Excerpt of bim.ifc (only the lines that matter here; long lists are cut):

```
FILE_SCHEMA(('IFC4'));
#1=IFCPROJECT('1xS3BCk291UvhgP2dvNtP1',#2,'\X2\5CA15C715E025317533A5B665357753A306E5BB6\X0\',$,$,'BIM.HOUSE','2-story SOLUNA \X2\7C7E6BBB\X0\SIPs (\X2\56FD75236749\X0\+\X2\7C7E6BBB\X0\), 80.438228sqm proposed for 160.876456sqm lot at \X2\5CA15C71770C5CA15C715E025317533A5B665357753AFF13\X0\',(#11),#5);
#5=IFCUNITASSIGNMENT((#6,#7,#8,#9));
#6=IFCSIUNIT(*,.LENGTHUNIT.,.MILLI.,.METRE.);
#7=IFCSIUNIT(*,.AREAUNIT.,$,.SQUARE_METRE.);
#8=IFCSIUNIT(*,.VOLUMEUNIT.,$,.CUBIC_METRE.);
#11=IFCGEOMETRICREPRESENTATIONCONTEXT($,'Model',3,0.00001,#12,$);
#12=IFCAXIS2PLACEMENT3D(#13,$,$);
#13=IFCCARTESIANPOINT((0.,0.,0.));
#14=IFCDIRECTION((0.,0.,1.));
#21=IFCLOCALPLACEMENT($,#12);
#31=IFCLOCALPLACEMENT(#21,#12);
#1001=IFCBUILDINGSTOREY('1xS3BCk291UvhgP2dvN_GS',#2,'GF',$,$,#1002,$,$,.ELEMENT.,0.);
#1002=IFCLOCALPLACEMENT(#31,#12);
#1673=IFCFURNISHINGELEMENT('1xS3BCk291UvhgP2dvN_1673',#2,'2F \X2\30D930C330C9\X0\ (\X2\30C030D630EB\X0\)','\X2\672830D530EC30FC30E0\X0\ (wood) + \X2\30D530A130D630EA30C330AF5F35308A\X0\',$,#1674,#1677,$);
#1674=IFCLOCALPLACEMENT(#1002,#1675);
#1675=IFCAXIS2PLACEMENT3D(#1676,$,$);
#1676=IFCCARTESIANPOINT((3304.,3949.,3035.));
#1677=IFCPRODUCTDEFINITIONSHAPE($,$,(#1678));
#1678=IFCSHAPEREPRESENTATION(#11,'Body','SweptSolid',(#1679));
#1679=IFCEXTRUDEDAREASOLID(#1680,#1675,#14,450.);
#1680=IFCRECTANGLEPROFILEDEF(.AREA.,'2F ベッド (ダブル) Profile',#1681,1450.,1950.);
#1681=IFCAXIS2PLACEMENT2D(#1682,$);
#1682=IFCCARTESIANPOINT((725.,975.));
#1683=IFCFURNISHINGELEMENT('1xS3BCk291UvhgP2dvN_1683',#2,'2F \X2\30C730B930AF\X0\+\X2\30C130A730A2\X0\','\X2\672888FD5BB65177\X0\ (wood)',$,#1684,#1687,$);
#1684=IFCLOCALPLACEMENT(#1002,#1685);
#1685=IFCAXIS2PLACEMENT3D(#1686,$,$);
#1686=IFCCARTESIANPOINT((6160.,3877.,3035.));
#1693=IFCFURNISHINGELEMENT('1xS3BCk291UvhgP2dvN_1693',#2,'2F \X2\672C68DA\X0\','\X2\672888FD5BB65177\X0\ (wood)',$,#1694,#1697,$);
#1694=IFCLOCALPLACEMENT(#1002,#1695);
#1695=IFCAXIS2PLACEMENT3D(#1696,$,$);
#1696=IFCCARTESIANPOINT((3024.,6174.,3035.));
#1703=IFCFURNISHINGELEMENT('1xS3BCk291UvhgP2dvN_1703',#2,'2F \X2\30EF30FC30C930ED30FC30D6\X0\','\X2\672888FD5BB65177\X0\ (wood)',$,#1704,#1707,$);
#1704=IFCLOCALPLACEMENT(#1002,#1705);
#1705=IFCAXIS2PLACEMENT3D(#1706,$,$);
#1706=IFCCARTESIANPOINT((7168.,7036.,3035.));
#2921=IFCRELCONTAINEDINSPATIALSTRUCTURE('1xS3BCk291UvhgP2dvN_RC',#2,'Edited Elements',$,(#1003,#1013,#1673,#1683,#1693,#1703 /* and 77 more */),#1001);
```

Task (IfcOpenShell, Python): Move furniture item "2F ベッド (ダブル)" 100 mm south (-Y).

```python
import ifcopenshell
import ifcopenshell.api.geometry
import ifcopenshell.util.placement
import ifcopenshell.util.unit

model = ifcopenshell.open("bim.ifc")
unit_scale = ifcopenshell.util.unit.calculate_unit_scale(model)

item = model.by_guid("1xS3BCk291UvhgP2dvN_1673")
matrix = ifcopenshell.util.placement.get_local_placement(item.ObjectPlacement)
matrix[1, 3] -= 0.1 / unit_scale
ifcopenshell.api.geometry.edit_object_placement(model, product=item, matrix=matrix, is_si=False)

print(ifcopenshell.util.placement.get_local_placement(item.ObjectPlacement).round(3) + 0.0)

model.write("bim_v2.ifc")
```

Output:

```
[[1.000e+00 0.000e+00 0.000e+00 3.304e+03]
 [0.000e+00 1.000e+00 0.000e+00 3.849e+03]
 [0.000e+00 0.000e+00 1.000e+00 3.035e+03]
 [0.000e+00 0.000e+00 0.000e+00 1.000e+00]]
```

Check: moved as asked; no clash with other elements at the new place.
